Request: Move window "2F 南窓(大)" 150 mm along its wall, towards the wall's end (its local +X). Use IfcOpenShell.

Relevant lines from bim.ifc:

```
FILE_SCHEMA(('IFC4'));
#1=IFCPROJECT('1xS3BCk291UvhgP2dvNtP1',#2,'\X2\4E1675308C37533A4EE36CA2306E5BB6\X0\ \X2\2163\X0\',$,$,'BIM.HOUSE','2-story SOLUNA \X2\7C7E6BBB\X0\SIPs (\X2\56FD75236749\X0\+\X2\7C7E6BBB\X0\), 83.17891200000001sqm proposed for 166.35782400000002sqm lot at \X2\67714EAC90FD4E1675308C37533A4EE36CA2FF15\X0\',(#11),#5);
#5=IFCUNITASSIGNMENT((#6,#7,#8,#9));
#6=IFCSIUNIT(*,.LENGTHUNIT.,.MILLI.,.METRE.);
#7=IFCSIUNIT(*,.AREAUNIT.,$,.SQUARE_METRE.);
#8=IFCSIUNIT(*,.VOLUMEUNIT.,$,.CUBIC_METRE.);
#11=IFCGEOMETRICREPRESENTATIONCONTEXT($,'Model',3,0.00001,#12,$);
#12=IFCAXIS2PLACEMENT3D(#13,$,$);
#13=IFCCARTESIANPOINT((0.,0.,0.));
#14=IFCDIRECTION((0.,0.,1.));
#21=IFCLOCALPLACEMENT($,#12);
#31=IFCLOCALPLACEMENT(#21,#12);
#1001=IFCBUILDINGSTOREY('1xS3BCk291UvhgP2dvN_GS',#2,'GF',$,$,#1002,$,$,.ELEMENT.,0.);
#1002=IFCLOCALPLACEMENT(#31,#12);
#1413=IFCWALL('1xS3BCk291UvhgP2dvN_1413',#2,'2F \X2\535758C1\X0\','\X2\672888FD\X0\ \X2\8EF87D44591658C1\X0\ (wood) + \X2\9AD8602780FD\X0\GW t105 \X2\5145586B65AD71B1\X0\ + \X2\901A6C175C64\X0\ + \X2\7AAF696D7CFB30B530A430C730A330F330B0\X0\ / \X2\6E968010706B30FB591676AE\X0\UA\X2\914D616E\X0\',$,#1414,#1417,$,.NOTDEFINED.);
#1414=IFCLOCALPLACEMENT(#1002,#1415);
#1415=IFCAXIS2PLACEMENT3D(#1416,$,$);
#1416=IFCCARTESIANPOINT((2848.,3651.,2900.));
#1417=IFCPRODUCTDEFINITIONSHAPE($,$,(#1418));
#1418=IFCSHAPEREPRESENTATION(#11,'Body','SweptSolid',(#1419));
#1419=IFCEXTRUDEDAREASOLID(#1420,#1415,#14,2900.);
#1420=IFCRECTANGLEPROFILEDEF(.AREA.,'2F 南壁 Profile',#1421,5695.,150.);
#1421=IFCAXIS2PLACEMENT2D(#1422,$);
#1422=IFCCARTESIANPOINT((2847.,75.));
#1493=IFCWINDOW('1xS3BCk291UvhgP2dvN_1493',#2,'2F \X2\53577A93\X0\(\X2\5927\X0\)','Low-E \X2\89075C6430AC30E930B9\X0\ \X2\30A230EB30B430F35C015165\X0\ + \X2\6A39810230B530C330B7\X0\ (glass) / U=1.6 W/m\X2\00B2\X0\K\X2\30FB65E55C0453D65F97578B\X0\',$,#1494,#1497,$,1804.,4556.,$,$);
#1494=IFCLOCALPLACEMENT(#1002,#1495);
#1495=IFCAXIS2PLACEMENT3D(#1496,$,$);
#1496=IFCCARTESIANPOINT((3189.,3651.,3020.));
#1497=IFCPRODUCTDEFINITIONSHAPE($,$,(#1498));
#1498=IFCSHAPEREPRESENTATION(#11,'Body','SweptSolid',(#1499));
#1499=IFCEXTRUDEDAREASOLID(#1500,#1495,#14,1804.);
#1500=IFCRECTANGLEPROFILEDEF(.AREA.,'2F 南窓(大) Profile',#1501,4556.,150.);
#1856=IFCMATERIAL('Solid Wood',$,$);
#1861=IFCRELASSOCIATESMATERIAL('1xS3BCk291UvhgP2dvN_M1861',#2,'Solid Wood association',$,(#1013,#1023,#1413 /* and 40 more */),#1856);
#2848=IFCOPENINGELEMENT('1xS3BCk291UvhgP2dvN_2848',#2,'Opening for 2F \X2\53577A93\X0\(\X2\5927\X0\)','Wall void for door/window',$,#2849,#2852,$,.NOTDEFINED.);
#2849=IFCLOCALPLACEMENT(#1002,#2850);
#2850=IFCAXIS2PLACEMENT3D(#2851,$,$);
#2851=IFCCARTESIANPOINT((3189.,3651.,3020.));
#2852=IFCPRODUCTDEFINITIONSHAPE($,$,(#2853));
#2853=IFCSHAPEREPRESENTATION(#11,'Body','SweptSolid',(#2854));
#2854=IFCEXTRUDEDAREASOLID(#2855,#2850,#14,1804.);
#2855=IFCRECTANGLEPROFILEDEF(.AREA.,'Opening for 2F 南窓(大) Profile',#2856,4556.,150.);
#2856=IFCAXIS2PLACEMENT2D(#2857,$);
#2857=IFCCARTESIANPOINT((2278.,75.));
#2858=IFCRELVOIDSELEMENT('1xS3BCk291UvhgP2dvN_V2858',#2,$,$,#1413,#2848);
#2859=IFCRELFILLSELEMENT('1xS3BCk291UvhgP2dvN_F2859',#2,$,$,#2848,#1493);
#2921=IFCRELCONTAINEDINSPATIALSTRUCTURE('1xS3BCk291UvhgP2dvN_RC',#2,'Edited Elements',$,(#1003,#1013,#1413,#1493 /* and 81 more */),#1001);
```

```python
import ifcopenshell
import ifcopenshell.api.geometry
import ifcopenshell.util.placement
import ifcopenshell.util.unit

model = ifcopenshell.open("bim.ifc")
unit_scale = ifcopenshell.util.unit.calculate_unit_scale(model)

window = model.by_id(1493)
opening = window.FillsVoids[0].RelatingOpeningElement
wall = opening.VoidsElements[0].RelatingBuildingElement

wall_matrix = ifcopenshell.util.placement.get_local_placement(wall.ObjectPlacement)
shift = wall_matrix[:3, 0] * 0.15 / unit_scale
before = ifcopenshell.util.placement.get_local_placement(window.ObjectPlacement)[:3, 3].copy()

# The window is not placed relative to its opening, so move both.
for product in (opening, window):
    matrix = ifcopenshell.util.placement.get_local_placement(product.ObjectPlacement)
    matrix[:3, 3] += shift
    ifcopenshell.api.geometry.edit_object_placement(model, product=product, matrix=matrix, is_si=False)

after = ifcopenshell.util.placement.get_local_placement(window.ObjectPlacement)[:3, 3]
print("window moved by", (after - before).round(3) + 0.0)

model.write("bim_rev.ifc")
```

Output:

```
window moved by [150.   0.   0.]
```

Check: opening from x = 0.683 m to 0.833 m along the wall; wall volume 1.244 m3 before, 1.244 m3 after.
